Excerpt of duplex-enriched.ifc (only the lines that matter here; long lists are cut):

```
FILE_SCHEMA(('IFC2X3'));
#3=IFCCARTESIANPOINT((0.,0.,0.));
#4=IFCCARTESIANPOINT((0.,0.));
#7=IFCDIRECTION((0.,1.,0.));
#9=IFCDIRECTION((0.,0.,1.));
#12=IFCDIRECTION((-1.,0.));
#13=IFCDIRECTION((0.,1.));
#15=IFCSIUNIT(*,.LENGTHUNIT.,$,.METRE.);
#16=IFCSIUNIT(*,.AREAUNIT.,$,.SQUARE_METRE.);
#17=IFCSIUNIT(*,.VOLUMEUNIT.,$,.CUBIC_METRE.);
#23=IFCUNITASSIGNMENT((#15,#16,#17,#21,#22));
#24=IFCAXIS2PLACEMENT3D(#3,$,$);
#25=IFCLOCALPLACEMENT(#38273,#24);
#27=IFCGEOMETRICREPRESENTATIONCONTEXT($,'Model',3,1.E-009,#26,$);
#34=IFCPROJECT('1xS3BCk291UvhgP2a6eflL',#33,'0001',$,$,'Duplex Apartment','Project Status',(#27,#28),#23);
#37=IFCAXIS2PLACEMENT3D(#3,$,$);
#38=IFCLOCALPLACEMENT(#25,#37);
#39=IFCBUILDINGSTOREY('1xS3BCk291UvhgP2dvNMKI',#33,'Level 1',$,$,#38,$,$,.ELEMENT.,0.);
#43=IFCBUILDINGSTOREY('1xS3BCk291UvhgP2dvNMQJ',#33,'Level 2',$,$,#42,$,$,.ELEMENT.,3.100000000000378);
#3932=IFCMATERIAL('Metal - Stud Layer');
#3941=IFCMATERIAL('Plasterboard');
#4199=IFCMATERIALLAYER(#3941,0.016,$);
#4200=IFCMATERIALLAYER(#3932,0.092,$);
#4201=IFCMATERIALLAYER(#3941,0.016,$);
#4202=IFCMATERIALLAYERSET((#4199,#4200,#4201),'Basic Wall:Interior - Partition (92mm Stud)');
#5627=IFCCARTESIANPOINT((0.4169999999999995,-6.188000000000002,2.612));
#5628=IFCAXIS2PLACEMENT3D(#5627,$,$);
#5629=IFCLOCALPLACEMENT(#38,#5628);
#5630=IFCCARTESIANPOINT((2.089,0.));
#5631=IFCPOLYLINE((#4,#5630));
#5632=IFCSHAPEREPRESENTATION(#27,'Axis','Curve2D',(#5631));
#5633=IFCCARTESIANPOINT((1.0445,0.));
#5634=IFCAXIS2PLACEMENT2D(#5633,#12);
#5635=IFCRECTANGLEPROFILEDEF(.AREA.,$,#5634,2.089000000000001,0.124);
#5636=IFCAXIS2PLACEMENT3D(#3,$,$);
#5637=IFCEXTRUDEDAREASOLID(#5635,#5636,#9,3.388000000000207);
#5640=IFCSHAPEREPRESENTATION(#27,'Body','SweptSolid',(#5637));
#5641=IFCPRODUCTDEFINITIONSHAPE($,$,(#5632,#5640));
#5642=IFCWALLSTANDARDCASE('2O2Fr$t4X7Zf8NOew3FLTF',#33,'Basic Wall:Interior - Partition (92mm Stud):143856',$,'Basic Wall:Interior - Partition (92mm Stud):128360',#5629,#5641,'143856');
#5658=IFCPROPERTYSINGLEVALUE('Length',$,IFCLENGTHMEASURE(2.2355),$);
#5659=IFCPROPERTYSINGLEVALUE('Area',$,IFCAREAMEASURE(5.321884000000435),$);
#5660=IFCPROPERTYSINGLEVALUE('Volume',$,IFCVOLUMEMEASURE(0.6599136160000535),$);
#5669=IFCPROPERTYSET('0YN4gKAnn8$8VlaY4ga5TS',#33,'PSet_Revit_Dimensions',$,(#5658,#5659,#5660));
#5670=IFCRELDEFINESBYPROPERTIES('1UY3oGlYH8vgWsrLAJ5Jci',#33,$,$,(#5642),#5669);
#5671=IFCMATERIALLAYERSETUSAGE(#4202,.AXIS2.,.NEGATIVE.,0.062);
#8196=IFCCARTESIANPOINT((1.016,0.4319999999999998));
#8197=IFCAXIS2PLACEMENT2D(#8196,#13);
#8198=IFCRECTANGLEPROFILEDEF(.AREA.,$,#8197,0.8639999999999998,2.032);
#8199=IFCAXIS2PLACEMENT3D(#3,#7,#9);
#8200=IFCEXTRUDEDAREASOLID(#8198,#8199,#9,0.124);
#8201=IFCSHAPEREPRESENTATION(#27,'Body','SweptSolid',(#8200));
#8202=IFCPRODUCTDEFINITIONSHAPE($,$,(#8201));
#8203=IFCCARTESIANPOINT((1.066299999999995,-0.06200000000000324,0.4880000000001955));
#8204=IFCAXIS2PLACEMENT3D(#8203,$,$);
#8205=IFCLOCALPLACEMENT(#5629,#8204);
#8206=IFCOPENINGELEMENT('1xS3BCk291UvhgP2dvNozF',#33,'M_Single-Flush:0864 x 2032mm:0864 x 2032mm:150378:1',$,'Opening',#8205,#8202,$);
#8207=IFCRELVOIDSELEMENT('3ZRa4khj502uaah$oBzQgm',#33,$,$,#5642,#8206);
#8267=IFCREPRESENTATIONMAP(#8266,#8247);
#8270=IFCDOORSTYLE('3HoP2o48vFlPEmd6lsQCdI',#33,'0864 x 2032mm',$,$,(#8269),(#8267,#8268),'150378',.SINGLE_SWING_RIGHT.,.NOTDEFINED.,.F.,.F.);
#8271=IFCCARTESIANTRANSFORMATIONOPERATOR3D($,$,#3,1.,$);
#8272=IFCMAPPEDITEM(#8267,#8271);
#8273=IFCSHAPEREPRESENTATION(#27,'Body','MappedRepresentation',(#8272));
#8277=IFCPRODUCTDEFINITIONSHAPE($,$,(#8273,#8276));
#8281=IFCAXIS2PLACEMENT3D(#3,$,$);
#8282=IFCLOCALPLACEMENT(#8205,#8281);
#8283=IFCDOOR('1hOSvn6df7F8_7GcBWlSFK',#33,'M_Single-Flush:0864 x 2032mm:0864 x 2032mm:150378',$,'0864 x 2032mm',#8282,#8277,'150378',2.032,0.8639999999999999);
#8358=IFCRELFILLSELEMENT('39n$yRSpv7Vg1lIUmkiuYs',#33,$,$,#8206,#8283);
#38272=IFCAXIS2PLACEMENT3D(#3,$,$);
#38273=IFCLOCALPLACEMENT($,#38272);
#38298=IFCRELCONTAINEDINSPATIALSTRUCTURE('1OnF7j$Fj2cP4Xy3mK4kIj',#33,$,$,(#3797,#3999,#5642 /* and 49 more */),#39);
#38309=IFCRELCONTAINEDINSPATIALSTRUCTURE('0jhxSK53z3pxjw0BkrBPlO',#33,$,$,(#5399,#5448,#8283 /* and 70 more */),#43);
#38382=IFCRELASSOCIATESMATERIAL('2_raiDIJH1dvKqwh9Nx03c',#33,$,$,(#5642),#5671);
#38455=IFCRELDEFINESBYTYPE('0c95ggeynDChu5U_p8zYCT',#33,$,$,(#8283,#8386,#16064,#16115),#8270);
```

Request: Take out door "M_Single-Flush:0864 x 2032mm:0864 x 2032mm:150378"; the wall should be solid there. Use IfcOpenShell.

```python
import ifcopenshell
import ifcopenshell.api.feature
import ifcopenshell.api.pset
import ifcopenshell.api.root
import ifcopenshell.geom
import ifcopenshell.util.element
import ifcopenshell.util.shape
import ifcopenshell.util.unit

model = ifcopenshell.open("duplex-enriched.ifc")
area_scale = ifcopenshell.util.unit.calculate_unit_scale(model, "AREAUNIT")
volume_scale = ifcopenshell.util.unit.calculate_unit_scale(model, "VOLUMEUNIT")
settings = ifcopenshell.geom.settings()


def volume(element):
    """Net volume in cubic metres, openings subtracted."""
    shape = ifcopenshell.geom.create_shape(settings, element)
    return ifcopenshell.util.shape.get_volume(shape.geometry)


door = model.by_guid("1hOSvn6df7F8_7GcBWlSFK")
opening = door.FillsVoids[0].RelatingOpeningElement
wall = opening.VoidsElements[0].RelatingBuildingElement
before = volume(wall)

ifcopenshell.api.root.remove_product(model, product=door)
ifcopenshell.api.feature.remove_feature(model, feature=opening)

after = volume(wall)
thickness = 0.124  # wall thickness in metres

# Update the wall's stored quantities.
pset = model.by_id(ifcopenshell.util.element.get_pset(wall, "PSet_Revit_Dimensions", should_inherit=False)["id"])
ifcopenshell.api.pset.edit_pset(model, pset=pset, properties={
    "Area": model.create_entity("IfcAreaMeasure", after / thickness / area_scale),
    "Volume": model.create_entity("IfcVolumeMeasure", after / volume_scale),
})

print(f"wall volume {before:.3f} -> {after:.3f} m3")

model.write("duplex-enriched_v2.ifc")
```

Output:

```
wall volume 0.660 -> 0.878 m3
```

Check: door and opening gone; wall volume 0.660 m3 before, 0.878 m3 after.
